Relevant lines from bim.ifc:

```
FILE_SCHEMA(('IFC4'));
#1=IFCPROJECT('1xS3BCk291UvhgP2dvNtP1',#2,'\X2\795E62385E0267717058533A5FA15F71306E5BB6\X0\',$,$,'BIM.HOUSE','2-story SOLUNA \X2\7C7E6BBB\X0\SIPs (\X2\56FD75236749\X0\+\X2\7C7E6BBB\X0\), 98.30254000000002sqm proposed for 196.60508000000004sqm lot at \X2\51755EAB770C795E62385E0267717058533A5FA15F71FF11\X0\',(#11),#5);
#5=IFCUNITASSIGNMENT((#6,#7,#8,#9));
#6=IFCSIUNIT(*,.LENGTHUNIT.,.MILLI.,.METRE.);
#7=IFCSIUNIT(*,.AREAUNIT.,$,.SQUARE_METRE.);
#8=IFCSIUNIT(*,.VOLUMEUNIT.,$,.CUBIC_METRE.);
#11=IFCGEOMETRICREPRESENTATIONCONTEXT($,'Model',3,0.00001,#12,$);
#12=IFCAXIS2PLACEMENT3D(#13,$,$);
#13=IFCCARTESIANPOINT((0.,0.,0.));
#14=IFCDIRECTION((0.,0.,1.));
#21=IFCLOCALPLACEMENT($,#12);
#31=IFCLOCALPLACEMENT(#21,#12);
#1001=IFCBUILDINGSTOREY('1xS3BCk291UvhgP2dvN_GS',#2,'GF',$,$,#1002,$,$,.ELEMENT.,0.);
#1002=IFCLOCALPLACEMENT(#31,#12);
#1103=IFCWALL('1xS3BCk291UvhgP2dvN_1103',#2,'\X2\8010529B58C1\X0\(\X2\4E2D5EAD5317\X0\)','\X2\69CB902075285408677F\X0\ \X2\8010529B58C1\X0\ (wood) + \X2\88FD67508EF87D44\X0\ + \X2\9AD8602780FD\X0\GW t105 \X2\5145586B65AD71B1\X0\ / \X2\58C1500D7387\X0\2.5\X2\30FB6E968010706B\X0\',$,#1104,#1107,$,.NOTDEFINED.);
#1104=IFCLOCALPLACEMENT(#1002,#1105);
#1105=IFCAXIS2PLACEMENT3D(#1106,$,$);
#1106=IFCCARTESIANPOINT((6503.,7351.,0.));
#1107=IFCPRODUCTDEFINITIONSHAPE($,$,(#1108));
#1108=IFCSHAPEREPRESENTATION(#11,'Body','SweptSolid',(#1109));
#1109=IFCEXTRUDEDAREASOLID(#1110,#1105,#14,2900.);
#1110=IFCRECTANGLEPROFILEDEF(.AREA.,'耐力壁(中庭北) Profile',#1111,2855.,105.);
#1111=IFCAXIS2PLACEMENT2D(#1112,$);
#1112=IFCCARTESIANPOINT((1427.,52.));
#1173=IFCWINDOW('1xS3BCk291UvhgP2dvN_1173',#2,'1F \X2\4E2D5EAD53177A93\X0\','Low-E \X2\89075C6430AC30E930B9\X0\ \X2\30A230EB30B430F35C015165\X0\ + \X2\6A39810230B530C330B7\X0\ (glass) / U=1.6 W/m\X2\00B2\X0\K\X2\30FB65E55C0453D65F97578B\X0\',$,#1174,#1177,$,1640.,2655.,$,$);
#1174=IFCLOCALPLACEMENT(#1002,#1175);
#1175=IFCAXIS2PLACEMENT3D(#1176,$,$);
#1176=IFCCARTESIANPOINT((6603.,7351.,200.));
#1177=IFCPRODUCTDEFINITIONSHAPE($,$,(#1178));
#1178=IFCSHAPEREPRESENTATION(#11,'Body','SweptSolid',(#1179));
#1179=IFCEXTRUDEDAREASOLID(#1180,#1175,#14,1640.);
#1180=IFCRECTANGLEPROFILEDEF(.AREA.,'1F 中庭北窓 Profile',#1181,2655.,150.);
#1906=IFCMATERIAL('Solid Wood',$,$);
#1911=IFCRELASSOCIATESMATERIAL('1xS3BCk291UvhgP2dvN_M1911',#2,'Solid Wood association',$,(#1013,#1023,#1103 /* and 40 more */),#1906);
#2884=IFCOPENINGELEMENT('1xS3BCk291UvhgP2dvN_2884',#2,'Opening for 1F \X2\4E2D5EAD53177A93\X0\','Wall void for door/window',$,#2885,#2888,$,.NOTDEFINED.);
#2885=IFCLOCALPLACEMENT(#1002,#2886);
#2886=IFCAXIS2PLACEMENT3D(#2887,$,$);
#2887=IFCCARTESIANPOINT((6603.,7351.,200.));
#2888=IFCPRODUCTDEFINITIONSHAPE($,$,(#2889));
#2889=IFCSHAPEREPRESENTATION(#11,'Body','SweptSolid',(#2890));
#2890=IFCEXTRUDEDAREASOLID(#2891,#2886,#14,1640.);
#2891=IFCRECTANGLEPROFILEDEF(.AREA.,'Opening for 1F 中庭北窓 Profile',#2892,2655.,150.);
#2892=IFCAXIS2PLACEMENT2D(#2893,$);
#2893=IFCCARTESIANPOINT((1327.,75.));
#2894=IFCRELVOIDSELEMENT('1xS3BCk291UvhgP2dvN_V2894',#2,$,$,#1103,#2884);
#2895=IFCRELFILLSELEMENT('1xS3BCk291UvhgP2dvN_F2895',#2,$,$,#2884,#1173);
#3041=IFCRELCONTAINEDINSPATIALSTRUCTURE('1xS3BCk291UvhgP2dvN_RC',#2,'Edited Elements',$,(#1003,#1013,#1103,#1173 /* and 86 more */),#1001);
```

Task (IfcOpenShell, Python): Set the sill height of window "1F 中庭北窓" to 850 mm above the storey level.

```python
import numpy as np
import ifcopenshell
import ifcopenshell.api.geometry
import ifcopenshell.geom
import ifcopenshell.util.element
import ifcopenshell.util.placement
import ifcopenshell.util.shape
import ifcopenshell.util.unit

model = ifcopenshell.open("bim.ifc")
unit_scale = ifcopenshell.util.unit.calculate_unit_scale(model)

window = model.by_guid("1xS3BCk291UvhgP2dvN_1173")
opening = window.FillsVoids[0].RelatingOpeningElement
storey = ifcopenshell.util.element.get_container(window, ifc_class="IfcBuildingStorey")
level = ifcopenshell.util.placement.get_local_placement(storey.ObjectPlacement)[2, 3]

# The opening's origin need not be at the sill, so measure its lowest point.
shape = ifcopenshell.geom.create_shape(ifcopenshell.geom.settings(), opening)
bottom = ifcopenshell.util.shape.get_shape_bottom_elevation(shape, shape.geometry) / unit_scale
dz = level + 850.0 - bottom

shift = np.array([0.0, 0.0, dz])
# The window is not placed relative to its opening, so move both.
for product in (opening, window):
    matrix = ifcopenshell.util.placement.get_local_placement(product.ObjectPlacement)
    matrix[:3, 3] += shift
    ifcopenshell.api.geometry.edit_object_placement(model, product=product, matrix=matrix, is_si=False)

print(f"moved by {dz * unit_scale:+.3f} m")

model.write("bim-out.ifc")
```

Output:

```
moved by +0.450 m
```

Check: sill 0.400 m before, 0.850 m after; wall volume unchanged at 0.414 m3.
